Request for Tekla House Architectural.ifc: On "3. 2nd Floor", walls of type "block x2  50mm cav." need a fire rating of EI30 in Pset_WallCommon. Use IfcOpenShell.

First a look at what the model holds.

```python
import ifcopenshell
import ifcopenshell.util.element

model = ifcopenshell.open("Tekla House Architectural.ifc")
print(model.schema)
storey = next(s for s in model.by_type("IfcBuildingStorey") if s.Name == "3. 2nd Floor")
walls = [e for e in ifcopenshell.util.element.get_decomposition(storey) if e.is_a("IfcWall")]
seen = {}
for e in walls:
    element_type = ifcopenshell.util.element.get_type(e)
    key = (element_type.Name if element_type != e and element_type else None, ifcopenshell.util.element.get_pset(e, "Pset_WallCommon", "FireRating"))
    seen[key] = seen.get(key, 0) + 1
for (name, value), count in sorted(seen.items(), key=str):
    print(count, "x", name, "|", value)
```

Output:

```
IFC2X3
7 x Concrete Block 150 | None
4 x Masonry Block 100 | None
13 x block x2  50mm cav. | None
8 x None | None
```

```python
import ifcopenshell
import ifcopenshell.api.pset
import ifcopenshell.util.element

model = ifcopenshell.open("Tekla House Architectural.ifc")

storey = next(s for s in model.by_type("IfcBuildingStorey") if s.Name == "3. 2nd Floor")
walls = [e for e in ifcopenshell.util.element.get_decomposition(storey) if e.is_a("IfcWall")]

count = 0
for e in walls:
    element_type = ifcopenshell.util.element.get_type(e)
    if element_type in (None, e) or element_type.Name != "block x2  50mm cav.":
        continue
    # add_pset returns the element's existing set when there is one.
    pset = ifcopenshell.api.pset.add_pset(model, product=e, name="Pset_WallCommon")
    ifcopenshell.api.pset.edit_pset(model, pset=pset, properties={"FireRating": "EI30"})
    count += 1

print(count, "walls updated")

model.write("Tekla House Architectural_rev.ifc")
```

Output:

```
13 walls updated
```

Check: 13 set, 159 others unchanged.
